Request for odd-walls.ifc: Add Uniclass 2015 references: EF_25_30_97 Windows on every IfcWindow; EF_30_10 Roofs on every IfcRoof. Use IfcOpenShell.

First a look at what the model holds.

```python
import ifcopenshell

model = ifcopenshell.open("odd-walls.ifc")
print(model.schema)
print("classifications:", [c.Name for c in model.by_type("IfcClassification")])
for ifc_class in ("IfcDoor", "IfcRoof", "IfcStair", "IfcWall", "IfcWindow"):
    print(ifc_class, len(model.by_type(ifc_class)))
```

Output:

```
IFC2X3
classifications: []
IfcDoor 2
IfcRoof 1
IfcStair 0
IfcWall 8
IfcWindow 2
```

```python
import ifcopenshell
import ifcopenshell.api.classification

model = ifcopenshell.open("odd-walls.ifc")

# IFC2X3 requires Source and Edition and has no link from the project to the system.
system = model.create_entity("IfcClassification", Source="NBS", Edition="2015", Name="Uniclass 2015")

codes = {
    "IfcWindow": ("EF_25_30_97", "Windows"),
    "IfcRoof": ("EF_30_10", "Roofs"),
}
for ifc_class, (code, name) in codes.items():
    products = model.by_type(ifc_class)
    ifcopenshell.api.classification.add_reference(
        model, products=products, classification=system, identification=code, name=name
    )
    print(code, len(products))

model.write("odd-walls-out.ifc")
```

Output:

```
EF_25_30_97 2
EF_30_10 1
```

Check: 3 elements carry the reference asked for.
